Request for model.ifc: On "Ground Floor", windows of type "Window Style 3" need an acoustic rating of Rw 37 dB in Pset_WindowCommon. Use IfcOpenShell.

First a look at what the model holds.

```python
import ifcopenshell
import ifcopenshell.util.element

model = ifcopenshell.open("model.ifc")
print(model.schema)
storey = next(s for s in model.by_type("IfcBuildingStorey") if s.Name == "Ground Floor")
windows = [e for e in ifcopenshell.util.element.get_decomposition(storey) if e.is_a("IfcWindow")]
seen = {}
for e in windows:
    element_type = ifcopenshell.util.element.get_type(e)
    key = (element_type.Name if element_type != e and element_type else None, ifcopenshell.util.element.get_pset(e, "Pset_WindowCommon", "AcousticRating"))
    seen[key] = seen.get(key, 0) + 1
for (name, value), count in sorted(seen.items(), key=str):
    print(count, "x", name, "|", value)
```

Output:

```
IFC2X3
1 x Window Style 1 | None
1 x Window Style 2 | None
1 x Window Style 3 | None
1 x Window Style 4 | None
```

```python
import ifcopenshell
import ifcopenshell.api.pset
import ifcopenshell.util.element

model = ifcopenshell.open("model.ifc")

storey = next(s for s in model.by_type("IfcBuildingStorey") if s.Name == "Ground Floor")
windows = [e for e in ifcopenshell.util.element.get_decomposition(storey) if e.is_a("IfcWindow")]

count = 0
for e in windows:
    element_type = ifcopenshell.util.element.get_type(e)
    if element_type in (None, e) or element_type.Name != "Window Style 3":
        continue
    # add_pset returns the element's existing set when there is one.
    pset = ifcopenshell.api.pset.add_pset(model, product=e, name="Pset_WindowCommon")
    ifcopenshell.api.pset.edit_pset(model, pset=pset, properties={"AcousticRating": "Rw 37 dB"})
    count += 1

print(count, "windows updated")

model.write("model_rev.ifc")
```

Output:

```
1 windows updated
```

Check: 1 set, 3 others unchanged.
